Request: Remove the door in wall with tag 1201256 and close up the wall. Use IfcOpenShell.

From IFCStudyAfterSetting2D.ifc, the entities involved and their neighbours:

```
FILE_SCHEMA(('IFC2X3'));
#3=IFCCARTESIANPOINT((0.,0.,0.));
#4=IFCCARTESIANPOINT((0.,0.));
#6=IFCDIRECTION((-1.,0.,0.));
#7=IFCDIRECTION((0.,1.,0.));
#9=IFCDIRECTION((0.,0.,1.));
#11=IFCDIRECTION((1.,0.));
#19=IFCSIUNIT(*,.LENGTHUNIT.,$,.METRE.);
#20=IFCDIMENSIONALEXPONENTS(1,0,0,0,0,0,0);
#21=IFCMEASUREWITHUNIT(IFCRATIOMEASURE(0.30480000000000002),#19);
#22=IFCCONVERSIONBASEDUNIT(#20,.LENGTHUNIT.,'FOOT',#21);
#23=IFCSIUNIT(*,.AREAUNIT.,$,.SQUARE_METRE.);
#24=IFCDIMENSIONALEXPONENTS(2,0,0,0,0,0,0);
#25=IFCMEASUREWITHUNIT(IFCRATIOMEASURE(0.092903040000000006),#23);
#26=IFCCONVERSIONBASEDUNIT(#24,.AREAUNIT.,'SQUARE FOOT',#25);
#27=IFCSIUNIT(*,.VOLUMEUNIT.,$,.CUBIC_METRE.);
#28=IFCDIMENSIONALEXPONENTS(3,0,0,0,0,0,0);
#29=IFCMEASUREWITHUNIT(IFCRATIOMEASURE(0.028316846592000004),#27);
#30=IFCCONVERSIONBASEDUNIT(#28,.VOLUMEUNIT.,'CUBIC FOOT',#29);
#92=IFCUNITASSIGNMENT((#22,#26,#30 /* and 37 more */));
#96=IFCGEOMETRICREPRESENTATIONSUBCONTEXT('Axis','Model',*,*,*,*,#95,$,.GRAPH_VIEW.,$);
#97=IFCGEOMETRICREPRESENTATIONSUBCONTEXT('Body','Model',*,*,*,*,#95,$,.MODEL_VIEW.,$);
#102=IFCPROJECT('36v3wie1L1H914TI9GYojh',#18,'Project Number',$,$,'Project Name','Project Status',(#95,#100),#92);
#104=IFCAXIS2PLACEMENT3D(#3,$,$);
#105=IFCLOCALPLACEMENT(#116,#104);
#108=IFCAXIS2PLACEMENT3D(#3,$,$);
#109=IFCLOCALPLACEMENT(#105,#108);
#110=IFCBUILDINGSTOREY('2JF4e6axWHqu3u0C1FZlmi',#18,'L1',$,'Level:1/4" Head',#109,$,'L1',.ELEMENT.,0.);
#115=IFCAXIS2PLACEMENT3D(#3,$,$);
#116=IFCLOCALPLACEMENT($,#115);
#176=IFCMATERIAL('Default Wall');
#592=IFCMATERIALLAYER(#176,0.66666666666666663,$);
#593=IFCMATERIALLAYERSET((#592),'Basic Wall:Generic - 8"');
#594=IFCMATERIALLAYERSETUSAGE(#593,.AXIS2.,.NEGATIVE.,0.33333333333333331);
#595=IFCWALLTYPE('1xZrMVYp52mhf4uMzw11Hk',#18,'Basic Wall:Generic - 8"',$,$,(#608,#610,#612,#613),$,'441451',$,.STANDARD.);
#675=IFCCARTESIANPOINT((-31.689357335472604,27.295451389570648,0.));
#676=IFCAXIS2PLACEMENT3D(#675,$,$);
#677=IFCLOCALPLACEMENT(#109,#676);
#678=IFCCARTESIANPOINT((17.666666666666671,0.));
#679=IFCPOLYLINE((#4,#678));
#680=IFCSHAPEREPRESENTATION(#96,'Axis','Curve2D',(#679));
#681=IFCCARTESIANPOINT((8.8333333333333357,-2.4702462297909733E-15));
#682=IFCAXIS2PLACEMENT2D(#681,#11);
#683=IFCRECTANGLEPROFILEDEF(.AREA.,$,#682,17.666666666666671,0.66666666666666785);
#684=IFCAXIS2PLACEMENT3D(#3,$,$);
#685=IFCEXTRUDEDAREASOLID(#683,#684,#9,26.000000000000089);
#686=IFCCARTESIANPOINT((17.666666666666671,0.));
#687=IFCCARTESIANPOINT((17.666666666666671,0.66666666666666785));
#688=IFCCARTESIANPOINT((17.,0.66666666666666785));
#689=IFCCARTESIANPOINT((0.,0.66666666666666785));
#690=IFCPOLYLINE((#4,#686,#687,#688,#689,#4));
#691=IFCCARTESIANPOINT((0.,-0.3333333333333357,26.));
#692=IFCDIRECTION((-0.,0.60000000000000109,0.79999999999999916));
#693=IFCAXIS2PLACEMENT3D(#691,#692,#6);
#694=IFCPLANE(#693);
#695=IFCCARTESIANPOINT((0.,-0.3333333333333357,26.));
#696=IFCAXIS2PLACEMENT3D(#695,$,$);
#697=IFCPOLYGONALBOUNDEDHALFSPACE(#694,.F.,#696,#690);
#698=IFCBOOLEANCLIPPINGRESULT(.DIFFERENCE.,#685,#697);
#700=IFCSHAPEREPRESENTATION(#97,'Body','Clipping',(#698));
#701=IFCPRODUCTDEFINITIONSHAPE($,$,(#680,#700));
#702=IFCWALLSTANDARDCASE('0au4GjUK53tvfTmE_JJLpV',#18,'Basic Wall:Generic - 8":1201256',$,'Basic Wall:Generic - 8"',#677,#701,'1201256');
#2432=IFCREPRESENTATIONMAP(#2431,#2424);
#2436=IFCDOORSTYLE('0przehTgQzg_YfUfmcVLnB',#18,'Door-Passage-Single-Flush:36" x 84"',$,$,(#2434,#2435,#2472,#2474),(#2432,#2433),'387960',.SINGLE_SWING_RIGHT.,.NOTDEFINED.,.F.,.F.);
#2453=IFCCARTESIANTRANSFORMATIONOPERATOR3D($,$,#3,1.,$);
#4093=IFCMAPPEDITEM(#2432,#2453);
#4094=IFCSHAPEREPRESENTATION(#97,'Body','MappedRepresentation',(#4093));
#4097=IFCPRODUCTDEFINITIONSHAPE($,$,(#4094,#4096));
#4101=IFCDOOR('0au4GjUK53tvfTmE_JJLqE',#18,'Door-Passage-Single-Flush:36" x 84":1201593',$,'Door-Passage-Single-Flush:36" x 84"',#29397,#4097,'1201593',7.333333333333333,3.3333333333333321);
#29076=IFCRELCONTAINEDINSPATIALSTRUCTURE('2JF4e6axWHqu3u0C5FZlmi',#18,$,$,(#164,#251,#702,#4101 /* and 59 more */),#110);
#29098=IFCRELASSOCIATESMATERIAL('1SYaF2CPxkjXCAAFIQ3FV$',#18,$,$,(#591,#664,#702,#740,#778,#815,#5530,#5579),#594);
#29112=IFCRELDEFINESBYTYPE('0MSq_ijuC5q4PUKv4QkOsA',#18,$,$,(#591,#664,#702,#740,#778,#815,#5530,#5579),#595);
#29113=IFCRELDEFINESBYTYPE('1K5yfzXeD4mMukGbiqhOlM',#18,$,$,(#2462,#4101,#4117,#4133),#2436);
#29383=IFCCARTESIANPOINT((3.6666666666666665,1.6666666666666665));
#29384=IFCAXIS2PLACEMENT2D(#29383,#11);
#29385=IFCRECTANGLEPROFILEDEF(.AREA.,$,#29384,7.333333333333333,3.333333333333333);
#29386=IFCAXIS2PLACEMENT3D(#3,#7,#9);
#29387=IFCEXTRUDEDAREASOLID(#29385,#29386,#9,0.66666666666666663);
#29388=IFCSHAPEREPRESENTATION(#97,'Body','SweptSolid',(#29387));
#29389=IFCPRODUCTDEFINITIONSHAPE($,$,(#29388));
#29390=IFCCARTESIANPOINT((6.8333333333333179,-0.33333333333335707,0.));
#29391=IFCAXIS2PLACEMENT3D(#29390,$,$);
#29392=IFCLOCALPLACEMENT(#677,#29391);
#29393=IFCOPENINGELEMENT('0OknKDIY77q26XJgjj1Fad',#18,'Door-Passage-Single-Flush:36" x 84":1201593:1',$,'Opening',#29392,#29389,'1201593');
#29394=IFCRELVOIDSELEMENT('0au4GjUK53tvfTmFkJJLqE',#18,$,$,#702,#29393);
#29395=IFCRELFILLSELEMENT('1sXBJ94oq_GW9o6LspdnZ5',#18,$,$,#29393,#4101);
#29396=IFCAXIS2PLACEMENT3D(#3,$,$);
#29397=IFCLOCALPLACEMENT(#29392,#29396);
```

```python
import ifcopenshell
import ifcopenshell.api.feature
import ifcopenshell.api.root
import ifcopenshell.geom
import ifcopenshell.util.shape

model = ifcopenshell.open("IFCStudyAfterSetting2D.ifc")
settings = ifcopenshell.geom.settings()


def volume(element):
    """Net volume in cubic metres, openings subtracted."""
    shape = ifcopenshell.geom.create_shape(settings, element)
    return ifcopenshell.util.shape.get_volume(shape.geometry)


door = model.by_guid("0au4GjUK53tvfTmE_JJLqE")
opening = door.FillsVoids[0].RelatingOpeningElement
wall = opening.VoidsElements[0].RelatingBuildingElement
before = volume(wall)

ifcopenshell.api.root.remove_product(model, product=door)
ifcopenshell.api.feature.remove_feature(model, feature=opening)

after = volume(wall)

print(f"wall volume {before:.3f} -> {after:.3f} m3")

model.write("IFCStudyAfterSetting2D_updated.ifc")
```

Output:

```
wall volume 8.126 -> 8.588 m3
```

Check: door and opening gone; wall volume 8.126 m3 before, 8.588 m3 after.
